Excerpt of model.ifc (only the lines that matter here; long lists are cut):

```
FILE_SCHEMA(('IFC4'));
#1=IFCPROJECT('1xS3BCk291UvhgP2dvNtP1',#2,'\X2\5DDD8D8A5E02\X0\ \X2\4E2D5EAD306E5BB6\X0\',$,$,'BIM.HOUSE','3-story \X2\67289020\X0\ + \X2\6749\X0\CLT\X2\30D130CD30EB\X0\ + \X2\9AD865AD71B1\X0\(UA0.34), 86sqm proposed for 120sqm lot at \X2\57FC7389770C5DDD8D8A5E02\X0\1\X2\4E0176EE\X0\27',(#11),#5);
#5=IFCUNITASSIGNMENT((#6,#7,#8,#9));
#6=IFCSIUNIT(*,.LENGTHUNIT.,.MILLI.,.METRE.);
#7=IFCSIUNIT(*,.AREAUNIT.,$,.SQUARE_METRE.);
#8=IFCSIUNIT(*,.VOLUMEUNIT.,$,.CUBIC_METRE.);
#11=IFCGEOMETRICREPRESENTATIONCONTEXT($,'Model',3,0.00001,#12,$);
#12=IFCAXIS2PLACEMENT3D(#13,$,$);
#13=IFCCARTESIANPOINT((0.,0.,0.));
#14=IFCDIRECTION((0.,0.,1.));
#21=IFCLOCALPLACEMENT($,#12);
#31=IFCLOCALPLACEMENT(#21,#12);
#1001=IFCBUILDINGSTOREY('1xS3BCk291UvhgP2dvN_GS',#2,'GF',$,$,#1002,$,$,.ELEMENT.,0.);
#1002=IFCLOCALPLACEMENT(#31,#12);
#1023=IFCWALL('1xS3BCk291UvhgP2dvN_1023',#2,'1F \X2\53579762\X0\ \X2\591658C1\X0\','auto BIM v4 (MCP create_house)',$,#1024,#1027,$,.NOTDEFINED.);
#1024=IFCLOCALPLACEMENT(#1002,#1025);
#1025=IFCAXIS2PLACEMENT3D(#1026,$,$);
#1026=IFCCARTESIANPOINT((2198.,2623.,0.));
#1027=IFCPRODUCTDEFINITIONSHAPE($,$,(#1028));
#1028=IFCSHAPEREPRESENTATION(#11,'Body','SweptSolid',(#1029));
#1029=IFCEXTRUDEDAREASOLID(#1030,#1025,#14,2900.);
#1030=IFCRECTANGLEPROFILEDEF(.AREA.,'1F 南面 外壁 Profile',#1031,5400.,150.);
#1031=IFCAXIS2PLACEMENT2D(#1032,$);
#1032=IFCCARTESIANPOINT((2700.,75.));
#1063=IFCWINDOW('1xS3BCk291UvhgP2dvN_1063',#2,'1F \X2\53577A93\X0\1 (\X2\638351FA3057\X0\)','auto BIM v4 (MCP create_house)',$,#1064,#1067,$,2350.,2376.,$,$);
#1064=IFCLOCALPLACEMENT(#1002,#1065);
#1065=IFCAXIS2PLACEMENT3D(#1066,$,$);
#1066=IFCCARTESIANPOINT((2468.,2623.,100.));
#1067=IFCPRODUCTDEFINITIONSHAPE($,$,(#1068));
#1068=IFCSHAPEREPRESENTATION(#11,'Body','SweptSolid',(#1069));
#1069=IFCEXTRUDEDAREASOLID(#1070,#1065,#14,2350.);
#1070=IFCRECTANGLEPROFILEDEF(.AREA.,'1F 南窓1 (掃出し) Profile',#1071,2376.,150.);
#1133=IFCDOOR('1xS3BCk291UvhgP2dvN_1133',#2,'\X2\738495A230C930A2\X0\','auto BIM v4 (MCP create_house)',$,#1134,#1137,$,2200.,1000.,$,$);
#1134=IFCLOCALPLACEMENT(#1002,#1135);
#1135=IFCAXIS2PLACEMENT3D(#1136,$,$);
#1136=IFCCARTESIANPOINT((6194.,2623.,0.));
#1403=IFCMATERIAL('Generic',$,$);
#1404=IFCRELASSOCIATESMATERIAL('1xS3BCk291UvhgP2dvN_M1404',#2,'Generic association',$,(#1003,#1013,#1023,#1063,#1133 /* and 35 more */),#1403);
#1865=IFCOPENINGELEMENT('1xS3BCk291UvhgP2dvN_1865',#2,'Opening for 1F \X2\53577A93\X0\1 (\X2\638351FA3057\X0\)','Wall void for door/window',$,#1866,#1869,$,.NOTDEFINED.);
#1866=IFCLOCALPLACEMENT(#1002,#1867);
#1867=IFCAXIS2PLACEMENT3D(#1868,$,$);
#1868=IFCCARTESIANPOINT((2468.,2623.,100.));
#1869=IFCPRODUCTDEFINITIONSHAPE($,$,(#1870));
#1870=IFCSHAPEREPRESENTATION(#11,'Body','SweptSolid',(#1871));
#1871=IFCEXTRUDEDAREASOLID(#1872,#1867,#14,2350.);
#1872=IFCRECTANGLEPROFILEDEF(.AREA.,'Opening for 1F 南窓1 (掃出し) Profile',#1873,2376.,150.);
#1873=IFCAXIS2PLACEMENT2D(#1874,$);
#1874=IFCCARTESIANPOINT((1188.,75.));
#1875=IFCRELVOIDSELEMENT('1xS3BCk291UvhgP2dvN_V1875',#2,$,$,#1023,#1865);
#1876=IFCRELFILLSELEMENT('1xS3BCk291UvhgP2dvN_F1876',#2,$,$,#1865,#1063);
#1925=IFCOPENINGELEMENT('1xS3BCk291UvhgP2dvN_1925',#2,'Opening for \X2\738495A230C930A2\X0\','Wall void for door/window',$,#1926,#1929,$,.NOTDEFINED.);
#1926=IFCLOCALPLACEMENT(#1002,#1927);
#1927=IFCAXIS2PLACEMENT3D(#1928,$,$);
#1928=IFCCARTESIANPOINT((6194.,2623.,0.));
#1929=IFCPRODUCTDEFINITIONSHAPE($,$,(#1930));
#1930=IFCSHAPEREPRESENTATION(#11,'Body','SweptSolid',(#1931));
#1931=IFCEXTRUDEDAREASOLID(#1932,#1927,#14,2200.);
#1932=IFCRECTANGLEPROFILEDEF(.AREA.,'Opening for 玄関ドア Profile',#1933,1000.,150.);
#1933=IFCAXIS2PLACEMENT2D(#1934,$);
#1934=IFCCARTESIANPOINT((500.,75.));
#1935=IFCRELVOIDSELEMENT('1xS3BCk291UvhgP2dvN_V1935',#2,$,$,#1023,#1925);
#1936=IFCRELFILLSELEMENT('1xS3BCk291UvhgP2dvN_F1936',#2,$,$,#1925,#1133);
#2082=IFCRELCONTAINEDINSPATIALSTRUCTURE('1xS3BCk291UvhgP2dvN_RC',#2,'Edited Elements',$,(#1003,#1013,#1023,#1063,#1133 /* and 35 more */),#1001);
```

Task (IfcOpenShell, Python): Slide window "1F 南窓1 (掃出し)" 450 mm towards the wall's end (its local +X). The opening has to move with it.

```python
import ifcopenshell
import ifcopenshell.api.geometry
import ifcopenshell.util.placement

model = ifcopenshell.open("model.ifc")

window = model.by_guid("1xS3BCk291UvhgP2dvN_1063")
opening = window.FillsVoids[0].RelatingOpeningElement
wall = opening.VoidsElements[0].RelatingBuildingElement

wall_matrix = ifcopenshell.util.placement.get_local_placement(wall.ObjectPlacement)
shift = wall_matrix[:3, 0] * 450.0
before = ifcopenshell.util.placement.get_local_placement(window.ObjectPlacement)[:3, 3].copy()

# The window is not placed relative to its opening, so move both.
for product in (opening, window):
    matrix = ifcopenshell.util.placement.get_local_placement(product.ObjectPlacement)
    matrix[:3, 3] += shift
    ifcopenshell.api.geometry.edit_object_placement(model, product=product, matrix=matrix, is_si=False)

after = ifcopenshell.util.placement.get_local_placement(window.ObjectPlacement)[:3, 3]
print("window moved by", (after - before).round(3) + 0.0)

model.write("model_rev.ifc")
```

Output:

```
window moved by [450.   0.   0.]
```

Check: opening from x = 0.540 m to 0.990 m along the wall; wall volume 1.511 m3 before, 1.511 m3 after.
